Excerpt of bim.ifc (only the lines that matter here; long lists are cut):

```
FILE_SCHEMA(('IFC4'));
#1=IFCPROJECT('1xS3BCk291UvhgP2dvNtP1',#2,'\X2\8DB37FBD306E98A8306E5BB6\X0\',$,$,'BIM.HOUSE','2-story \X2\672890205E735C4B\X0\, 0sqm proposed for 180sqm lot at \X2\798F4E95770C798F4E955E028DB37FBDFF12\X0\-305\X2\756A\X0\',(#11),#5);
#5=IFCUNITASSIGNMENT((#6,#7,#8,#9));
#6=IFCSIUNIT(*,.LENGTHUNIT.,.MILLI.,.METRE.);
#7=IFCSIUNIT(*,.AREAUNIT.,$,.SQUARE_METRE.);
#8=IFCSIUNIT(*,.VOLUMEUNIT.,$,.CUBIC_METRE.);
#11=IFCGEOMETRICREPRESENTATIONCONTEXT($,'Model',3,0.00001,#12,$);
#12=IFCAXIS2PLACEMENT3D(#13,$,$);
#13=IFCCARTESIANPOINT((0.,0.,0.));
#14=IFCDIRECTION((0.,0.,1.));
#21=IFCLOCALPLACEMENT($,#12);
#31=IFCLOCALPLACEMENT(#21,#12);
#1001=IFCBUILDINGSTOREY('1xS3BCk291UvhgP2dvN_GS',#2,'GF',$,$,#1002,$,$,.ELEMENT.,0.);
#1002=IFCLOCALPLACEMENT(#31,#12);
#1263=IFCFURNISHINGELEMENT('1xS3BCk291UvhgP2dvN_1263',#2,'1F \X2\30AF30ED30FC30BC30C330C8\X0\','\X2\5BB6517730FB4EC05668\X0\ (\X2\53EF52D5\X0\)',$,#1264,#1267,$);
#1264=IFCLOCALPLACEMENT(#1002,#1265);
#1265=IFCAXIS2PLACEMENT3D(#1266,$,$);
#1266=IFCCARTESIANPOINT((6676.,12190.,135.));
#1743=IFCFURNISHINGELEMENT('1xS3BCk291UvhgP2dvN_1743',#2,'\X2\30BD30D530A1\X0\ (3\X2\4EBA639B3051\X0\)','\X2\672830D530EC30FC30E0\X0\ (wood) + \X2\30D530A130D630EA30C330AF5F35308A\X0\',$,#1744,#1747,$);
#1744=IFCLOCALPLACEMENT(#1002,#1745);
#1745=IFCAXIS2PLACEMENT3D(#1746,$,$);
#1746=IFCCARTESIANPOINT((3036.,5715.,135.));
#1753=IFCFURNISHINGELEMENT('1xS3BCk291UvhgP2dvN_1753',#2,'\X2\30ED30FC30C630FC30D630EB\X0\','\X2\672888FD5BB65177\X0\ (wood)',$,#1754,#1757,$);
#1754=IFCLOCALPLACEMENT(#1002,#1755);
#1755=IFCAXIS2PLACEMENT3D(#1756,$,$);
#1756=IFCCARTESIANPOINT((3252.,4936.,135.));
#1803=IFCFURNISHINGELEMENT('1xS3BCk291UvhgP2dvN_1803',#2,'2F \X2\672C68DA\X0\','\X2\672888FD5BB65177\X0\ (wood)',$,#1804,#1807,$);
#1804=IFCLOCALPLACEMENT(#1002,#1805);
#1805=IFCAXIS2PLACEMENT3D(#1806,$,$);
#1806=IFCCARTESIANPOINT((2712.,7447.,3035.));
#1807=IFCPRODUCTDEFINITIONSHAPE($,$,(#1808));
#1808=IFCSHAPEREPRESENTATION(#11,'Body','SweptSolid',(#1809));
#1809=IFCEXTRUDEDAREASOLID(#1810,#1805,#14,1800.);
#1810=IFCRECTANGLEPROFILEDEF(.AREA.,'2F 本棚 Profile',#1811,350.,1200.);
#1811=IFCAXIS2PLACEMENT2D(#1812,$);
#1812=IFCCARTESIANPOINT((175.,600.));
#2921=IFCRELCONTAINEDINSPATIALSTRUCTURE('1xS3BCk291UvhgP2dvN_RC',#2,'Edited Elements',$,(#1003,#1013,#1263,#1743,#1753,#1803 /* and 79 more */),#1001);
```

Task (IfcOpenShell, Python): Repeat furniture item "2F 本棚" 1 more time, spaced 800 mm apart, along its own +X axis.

```python
import ifcopenshell
import ifcopenshell.api.geometry
import ifcopenshell.api.root
import ifcopenshell.util.element
import ifcopenshell.util.placement

model = ifcopenshell.open("bim.ifc")


def reuse_history(source, copy):
    """copy_class also copies each property set's owner history, people and application; keep the originals."""
    for rel in copy.IsDefinedBy:
        if rel.is_a("IfcRelDefinesByProperties") and (history := rel.RelatingPropertyDefinition.OwnerHistory):
            rel.RelatingPropertyDefinition.OwnerHistory = source.OwnerHistory
            ifcopenshell.util.element.remove_deep2(model, history)


source = model.by_guid("1xS3BCk291UvhgP2dvN_1803")
base = ifcopenshell.util.placement.get_local_placement(source.ObjectPlacement)
step = base[:3, 0] * 800.0

for i in range(1, 2):
    copy = ifcopenshell.api.root.copy_class(model, product=source)
    copy.Representation = ifcopenshell.util.element.copy_deep(
        model, source.Representation, exclude=["IfcGeometricRepresentationContext", "IfcRepresentationMap"]
    )
    reuse_history(source, copy)
    matrix = base.copy()
    matrix[:3, 3] += i * step
    print("added at", matrix[:3, 3].round(3) + 0.0)
    ifcopenshell.api.geometry.edit_object_placement(model, product=copy, matrix=matrix, is_si=False)

model.write("bim_v2.ifc")
```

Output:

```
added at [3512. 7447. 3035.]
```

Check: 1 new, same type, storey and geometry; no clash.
